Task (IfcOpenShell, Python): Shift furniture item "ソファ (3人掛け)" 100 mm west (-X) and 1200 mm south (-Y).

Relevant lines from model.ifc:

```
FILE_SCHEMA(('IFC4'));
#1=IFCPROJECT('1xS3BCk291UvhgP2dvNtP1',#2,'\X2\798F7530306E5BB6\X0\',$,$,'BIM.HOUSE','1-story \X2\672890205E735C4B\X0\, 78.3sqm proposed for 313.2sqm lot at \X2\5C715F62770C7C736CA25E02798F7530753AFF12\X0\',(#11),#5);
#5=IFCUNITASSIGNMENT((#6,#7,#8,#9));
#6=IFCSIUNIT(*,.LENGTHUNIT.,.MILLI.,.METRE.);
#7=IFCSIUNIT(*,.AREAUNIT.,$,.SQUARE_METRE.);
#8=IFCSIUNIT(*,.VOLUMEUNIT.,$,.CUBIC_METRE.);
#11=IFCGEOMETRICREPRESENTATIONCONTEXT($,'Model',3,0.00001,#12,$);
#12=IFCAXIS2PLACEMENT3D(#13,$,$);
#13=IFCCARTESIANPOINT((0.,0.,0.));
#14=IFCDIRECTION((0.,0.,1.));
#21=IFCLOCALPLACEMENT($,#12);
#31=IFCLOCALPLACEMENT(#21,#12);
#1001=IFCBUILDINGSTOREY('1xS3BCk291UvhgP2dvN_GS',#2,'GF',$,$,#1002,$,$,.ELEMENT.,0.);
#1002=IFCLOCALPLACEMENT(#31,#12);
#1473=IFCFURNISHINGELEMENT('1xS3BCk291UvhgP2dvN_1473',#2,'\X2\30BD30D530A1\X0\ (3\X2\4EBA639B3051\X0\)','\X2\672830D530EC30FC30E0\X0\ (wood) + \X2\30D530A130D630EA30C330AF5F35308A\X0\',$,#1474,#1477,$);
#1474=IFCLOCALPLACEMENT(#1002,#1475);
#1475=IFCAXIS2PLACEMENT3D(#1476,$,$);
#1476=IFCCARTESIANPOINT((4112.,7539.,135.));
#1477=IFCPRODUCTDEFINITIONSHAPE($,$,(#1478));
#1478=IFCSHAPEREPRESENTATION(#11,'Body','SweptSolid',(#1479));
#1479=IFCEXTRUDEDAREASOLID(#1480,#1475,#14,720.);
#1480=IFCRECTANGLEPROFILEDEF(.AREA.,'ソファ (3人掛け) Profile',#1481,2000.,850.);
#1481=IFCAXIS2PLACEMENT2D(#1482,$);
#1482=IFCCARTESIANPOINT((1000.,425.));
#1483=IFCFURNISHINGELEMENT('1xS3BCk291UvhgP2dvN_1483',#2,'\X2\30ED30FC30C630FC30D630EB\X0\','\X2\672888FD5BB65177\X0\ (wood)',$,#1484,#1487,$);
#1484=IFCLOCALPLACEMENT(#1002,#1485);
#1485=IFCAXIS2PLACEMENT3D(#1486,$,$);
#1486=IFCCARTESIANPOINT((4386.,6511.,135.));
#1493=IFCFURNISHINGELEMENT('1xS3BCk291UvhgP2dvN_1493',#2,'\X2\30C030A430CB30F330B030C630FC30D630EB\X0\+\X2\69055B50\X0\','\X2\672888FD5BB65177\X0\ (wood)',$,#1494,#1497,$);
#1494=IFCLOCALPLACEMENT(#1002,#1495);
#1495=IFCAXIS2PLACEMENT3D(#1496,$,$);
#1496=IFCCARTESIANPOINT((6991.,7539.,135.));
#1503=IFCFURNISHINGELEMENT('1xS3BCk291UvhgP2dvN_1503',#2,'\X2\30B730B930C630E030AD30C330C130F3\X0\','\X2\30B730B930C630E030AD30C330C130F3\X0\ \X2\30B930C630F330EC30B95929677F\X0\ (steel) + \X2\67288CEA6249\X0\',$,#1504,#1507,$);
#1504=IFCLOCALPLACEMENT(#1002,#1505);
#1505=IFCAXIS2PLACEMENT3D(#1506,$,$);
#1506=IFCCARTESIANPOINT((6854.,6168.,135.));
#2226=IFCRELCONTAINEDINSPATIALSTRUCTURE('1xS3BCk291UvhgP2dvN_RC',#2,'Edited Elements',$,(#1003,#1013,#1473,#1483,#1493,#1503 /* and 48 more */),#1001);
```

```python
import ifcopenshell
import ifcopenshell.api.geometry
import ifcopenshell.util.placement

model = ifcopenshell.open("model.ifc")

item = model.by_guid("1xS3BCk291UvhgP2dvN_1473")
matrix = ifcopenshell.util.placement.get_local_placement(item.ObjectPlacement)
matrix[0, 3] -= 100.0
matrix[1, 3] -= 1200.0
ifcopenshell.api.geometry.edit_object_placement(model, product=item, matrix=matrix, is_si=False)

print(ifcopenshell.util.placement.get_local_placement(item.ObjectPlacement).round(3) + 0.0)

model.write("model_rev.ifc")
```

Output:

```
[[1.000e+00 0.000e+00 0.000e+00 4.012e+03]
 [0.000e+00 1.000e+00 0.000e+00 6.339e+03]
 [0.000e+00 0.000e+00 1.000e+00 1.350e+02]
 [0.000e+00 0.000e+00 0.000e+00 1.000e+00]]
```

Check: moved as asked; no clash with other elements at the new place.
